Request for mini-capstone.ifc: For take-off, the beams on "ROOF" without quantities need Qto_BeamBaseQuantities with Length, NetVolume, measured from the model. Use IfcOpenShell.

First a look at what the model holds.

```python
import ifcopenshell
import ifcopenshell.util.element
import ifcopenshell.util.unit

model = ifcopenshell.open("mini-capstone.ifc")
print(model.schema)
for unit_type in ("LENGTHUNIT", "AREAUNIT", "VOLUMEUNIT"):
    print(unit_type, ifcopenshell.util.unit.calculate_unit_scale(model, unit_type))
storey = next(s for s in model.by_type("IfcBuildingStorey") if s.Name == "ROOF")
beams = [e for e in ifcopenshell.util.element.get_decomposition(storey) if e.is_a("IfcBeam")]
for e in sorted(beams, key=lambda e: e.id()):
    print(e.id(), e.is_a(), e.Name, list(ifcopenshell.util.element.get_psets(e, qtos_only=True)), sep=" | ")
```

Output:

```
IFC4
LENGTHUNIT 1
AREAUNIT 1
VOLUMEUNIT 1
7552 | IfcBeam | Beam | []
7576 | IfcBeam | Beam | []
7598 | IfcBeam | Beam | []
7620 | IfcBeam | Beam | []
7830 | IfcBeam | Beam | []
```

```python
import ifcopenshell
import ifcopenshell.api.pset
import ifcopenshell.geom
import ifcopenshell.util.element
import ifcopenshell.util.shape
import ifcopenshell.util.unit

model = ifcopenshell.open("mini-capstone.ifc")
unit_scale = ifcopenshell.util.unit.calculate_unit_scale(model)
volume_scale = ifcopenshell.util.unit.calculate_unit_scale(model, "VOLUMEUNIT")
settings = ifcopenshell.geom.settings()

storey = next(s for s in model.by_type("IfcBuildingStorey") if s.Name == "ROOF")
beams = [e for e in ifcopenshell.util.element.get_decomposition(storey) if e.is_a("IfcBeam")]

for e in sorted(beams, key=lambda e: e.id()):
    if ifcopenshell.util.element.get_psets(e, qtos_only=True, should_inherit=False):
        continue
    # Geometry comes back in metres, in the element's own axes.
    shape = ifcopenshell.geom.create_shape(settings, e)
    values = {
        "Length": ifcopenshell.util.shape.get_max_xyz(shape.geometry) / unit_scale,
        "NetVolume": ifcopenshell.util.shape.get_volume(shape.geometry) / volume_scale,
    }
    qto = ifcopenshell.api.pset.add_qto(model, product=e, name="Qto_BeamBaseQuantities")
    ifcopenshell.api.pset.edit_qto(model, qto=qto, properties=values)
    print(e.id(), {k: round(v, 3) for k, v in values.items()})

model.write("mini-capstone_edited.ifc")
```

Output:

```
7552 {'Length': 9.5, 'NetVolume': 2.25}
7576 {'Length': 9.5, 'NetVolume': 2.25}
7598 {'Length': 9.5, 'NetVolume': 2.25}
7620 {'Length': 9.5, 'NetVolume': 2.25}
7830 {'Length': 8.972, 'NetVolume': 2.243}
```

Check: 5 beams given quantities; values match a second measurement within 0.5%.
